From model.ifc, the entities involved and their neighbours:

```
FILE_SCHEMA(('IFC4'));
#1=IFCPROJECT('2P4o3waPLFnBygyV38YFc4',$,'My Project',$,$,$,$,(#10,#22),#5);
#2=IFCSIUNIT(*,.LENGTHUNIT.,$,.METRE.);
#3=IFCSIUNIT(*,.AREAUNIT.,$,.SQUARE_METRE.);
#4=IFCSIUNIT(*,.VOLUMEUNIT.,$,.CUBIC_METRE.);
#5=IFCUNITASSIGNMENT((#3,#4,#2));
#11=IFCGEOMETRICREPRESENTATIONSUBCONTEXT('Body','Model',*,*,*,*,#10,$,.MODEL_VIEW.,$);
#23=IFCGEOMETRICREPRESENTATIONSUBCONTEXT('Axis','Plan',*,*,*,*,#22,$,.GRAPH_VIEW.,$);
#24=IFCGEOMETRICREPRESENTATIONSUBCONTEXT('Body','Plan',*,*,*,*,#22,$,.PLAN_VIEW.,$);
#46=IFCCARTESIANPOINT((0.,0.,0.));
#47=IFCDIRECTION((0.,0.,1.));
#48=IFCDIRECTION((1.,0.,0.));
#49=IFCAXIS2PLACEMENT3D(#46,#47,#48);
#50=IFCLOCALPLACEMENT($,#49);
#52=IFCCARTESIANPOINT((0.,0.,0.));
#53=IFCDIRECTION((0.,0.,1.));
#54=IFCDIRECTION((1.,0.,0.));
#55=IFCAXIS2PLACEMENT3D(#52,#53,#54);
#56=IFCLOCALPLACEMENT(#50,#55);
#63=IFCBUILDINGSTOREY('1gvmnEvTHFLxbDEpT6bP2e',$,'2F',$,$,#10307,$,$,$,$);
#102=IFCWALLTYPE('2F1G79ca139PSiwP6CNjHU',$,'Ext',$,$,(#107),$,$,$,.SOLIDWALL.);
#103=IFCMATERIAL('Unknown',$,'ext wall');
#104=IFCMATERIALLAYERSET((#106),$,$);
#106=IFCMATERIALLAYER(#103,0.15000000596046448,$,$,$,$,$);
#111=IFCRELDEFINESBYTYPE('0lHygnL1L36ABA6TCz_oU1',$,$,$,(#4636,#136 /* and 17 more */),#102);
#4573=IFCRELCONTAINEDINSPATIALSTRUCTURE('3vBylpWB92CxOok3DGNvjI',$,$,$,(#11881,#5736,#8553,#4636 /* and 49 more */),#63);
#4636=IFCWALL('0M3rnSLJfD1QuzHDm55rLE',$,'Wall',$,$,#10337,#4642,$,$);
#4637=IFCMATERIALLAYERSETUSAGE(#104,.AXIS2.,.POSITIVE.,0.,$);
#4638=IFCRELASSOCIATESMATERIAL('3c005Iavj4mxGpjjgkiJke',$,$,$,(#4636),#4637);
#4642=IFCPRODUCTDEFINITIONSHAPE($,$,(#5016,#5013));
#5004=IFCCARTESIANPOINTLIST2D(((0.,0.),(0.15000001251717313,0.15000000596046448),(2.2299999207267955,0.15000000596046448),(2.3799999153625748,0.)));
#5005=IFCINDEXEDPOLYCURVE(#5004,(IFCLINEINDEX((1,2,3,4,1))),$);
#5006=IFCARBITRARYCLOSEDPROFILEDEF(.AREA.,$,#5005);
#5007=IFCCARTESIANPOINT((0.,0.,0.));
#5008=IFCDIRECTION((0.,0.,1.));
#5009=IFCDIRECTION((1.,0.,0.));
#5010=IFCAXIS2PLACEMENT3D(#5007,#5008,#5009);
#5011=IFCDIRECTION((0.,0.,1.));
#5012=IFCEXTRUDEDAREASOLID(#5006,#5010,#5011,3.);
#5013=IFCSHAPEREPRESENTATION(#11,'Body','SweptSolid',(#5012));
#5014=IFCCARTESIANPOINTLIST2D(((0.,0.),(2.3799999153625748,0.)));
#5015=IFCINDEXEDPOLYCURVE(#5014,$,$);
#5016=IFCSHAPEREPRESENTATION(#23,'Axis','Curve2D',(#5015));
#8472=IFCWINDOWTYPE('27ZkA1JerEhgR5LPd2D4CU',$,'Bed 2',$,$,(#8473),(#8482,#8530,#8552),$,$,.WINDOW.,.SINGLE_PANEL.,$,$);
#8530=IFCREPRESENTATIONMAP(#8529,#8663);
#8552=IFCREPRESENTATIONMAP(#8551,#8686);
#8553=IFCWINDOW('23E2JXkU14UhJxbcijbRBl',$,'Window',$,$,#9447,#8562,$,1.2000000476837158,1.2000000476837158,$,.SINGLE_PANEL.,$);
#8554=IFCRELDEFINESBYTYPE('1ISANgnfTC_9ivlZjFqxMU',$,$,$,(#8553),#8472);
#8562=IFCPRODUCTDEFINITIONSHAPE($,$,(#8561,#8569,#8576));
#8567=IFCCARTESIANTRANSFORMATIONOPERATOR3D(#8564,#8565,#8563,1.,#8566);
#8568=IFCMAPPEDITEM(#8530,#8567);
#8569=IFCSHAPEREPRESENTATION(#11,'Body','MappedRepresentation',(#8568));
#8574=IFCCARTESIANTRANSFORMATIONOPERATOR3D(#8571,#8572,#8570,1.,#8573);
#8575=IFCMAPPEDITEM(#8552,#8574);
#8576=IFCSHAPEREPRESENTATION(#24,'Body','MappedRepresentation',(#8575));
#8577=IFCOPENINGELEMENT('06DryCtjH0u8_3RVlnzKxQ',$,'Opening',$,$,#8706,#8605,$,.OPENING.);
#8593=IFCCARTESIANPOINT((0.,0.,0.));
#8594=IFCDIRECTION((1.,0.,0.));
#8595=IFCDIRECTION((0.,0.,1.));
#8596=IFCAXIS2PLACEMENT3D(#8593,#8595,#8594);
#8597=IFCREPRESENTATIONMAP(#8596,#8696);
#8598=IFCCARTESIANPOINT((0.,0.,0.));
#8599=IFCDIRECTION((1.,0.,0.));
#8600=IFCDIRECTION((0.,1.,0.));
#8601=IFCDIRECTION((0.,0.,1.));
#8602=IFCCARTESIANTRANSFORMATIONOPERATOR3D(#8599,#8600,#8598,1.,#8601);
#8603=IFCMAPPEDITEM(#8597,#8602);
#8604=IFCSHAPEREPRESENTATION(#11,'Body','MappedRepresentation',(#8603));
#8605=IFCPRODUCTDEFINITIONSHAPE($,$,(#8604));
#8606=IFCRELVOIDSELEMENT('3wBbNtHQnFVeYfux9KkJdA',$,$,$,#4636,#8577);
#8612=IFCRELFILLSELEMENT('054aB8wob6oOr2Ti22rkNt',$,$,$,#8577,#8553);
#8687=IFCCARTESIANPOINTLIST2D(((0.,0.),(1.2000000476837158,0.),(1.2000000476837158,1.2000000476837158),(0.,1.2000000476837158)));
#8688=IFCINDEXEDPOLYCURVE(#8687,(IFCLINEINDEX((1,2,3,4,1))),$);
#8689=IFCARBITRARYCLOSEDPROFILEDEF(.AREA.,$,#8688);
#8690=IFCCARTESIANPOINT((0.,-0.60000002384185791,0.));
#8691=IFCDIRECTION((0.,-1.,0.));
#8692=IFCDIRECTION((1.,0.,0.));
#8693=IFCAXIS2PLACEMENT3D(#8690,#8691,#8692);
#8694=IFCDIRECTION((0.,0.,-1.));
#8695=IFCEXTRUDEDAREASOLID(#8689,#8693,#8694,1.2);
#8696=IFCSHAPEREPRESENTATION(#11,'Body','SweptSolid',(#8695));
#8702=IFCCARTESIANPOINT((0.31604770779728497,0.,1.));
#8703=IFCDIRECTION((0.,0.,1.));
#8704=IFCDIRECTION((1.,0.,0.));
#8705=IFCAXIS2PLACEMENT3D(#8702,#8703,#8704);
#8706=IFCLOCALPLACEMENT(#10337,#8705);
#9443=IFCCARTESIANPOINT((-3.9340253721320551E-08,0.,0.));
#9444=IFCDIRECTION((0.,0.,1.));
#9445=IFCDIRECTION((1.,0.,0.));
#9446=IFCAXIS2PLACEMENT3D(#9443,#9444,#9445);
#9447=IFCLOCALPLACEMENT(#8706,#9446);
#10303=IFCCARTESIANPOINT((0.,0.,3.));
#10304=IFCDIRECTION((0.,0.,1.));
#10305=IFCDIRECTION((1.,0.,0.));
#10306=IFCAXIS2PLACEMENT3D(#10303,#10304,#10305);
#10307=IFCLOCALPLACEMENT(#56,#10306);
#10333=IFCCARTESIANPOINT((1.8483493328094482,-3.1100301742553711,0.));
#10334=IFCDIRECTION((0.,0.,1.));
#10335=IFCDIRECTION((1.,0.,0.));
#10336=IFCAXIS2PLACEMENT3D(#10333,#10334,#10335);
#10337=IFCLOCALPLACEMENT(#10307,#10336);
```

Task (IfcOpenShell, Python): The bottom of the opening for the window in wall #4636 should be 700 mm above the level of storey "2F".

```python
import numpy as np
import ifcopenshell
import ifcopenshell.api.geometry
import ifcopenshell.geom
import ifcopenshell.util.element
import ifcopenshell.util.placement
import ifcopenshell.util.shape
import ifcopenshell.util.unit

model = ifcopenshell.open("model.ifc")
unit_scale = ifcopenshell.util.unit.calculate_unit_scale(model)

window = model.by_guid("23E2JXkU14UhJxbcijbRBl")
opening = window.FillsVoids[0].RelatingOpeningElement
storey = ifcopenshell.util.element.get_container(window, ifc_class="IfcBuildingStorey")
level = ifcopenshell.util.placement.get_local_placement(storey.ObjectPlacement)[2, 3]

# The opening's origin need not be at the sill, so measure its lowest point.
shape = ifcopenshell.geom.create_shape(ifcopenshell.geom.settings(), opening)
bottom = ifcopenshell.util.shape.get_shape_bottom_elevation(shape, shape.geometry) / unit_scale
dz = level + 0.7 / unit_scale - bottom

shift = np.array([0.0, 0.0, dz])
# The window is placed relative to its opening, so it follows when the opening moves.
matrix = ifcopenshell.util.placement.get_local_placement(opening.ObjectPlacement)
matrix[:3, 3] += shift
ifcopenshell.api.geometry.edit_object_placement(
    model, product=opening, matrix=matrix, is_si=False, should_transform_children=True
)

print(f"moved by {dz * unit_scale:+.3f} m")

model.write("model-out.ifc")
```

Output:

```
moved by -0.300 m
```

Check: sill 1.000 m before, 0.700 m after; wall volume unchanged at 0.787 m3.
